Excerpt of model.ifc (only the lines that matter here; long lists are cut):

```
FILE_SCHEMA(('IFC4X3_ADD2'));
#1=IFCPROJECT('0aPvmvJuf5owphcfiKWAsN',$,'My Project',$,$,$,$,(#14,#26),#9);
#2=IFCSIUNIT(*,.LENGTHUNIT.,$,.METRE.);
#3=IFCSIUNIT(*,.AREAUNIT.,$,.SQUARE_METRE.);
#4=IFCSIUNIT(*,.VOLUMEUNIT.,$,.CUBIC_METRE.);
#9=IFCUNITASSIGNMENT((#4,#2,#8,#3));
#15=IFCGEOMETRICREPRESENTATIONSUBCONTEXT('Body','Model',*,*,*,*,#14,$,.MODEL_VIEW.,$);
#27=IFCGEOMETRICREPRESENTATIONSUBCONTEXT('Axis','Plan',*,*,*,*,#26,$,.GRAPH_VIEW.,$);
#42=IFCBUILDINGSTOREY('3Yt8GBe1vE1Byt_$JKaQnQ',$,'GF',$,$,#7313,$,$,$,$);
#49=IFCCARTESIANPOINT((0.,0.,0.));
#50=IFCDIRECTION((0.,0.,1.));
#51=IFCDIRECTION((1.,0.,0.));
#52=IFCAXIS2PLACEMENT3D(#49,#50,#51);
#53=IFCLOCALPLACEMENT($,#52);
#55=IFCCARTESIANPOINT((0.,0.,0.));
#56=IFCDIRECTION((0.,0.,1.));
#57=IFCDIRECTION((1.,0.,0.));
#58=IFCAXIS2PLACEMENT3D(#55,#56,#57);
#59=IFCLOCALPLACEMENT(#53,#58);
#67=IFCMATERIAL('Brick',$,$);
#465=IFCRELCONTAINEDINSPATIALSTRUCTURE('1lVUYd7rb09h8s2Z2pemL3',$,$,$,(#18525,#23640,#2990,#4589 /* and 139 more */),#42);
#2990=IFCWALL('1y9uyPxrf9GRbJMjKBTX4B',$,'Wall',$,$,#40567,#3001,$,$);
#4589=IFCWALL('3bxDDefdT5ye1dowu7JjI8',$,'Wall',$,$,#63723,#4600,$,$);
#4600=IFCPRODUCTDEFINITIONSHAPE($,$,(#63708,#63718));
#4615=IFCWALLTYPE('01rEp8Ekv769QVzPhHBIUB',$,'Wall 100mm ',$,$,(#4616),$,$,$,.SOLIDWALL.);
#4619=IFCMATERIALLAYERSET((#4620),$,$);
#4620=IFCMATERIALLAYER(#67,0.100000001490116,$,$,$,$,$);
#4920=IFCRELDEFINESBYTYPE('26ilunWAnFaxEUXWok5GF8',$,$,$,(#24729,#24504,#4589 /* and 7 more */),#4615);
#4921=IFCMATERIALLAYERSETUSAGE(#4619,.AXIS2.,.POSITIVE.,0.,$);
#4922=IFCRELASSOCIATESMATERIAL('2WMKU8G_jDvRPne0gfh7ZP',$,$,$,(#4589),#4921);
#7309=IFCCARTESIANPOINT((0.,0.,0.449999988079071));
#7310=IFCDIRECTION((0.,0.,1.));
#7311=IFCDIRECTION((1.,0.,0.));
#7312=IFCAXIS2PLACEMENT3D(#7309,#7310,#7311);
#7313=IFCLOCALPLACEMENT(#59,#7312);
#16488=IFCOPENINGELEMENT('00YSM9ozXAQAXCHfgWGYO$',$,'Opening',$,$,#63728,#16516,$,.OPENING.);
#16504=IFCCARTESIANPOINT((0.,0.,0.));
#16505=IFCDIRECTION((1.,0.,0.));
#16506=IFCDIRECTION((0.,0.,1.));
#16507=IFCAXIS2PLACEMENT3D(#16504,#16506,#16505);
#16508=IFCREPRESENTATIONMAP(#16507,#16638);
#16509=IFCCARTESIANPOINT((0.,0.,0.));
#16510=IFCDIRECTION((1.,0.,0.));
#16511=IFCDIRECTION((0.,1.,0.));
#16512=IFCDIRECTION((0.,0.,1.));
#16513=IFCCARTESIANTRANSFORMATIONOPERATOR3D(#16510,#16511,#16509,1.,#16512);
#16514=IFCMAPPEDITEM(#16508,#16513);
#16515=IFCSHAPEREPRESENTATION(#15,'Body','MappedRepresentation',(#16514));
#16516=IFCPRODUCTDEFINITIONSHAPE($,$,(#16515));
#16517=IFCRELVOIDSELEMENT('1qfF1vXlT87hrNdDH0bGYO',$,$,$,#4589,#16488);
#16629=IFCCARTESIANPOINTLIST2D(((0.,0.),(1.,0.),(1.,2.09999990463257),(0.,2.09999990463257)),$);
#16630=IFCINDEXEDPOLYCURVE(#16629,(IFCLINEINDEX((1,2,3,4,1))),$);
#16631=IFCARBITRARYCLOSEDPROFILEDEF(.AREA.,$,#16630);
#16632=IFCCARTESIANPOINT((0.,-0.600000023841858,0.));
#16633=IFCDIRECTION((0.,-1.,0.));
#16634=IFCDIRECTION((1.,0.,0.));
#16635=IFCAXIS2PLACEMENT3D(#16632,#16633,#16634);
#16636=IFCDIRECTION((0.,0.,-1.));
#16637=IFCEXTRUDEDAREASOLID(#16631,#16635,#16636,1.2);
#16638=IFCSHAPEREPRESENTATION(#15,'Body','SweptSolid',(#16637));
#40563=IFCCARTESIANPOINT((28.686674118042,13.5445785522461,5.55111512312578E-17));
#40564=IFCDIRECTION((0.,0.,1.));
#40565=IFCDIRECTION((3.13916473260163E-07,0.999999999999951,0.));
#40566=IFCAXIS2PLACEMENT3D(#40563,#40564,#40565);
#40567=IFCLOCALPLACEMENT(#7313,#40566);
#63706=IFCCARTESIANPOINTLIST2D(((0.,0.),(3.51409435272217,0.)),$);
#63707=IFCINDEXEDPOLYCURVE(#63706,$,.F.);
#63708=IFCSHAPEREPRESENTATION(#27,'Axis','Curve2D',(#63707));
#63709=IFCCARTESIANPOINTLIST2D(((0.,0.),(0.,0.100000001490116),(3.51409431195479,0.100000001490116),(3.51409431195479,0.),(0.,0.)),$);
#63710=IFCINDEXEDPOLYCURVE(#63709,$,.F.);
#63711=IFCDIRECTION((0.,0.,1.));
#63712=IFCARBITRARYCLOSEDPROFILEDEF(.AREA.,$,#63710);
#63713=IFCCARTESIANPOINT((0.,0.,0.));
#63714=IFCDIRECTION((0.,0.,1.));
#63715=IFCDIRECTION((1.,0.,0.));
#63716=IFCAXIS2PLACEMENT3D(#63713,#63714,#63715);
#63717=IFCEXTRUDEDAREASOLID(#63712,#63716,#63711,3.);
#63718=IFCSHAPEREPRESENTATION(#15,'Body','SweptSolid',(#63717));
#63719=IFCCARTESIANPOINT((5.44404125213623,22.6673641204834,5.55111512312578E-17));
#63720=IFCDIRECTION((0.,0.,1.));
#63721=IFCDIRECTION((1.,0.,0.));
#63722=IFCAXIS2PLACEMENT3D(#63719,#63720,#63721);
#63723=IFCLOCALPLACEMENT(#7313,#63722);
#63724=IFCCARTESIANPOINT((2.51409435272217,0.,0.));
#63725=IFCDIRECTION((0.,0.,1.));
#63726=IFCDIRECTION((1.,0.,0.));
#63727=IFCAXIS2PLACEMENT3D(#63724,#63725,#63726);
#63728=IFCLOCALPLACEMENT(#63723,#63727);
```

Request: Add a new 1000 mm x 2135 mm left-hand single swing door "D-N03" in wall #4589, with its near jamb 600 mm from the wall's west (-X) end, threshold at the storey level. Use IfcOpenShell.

```python
import numpy as np
import ifcopenshell
import ifcopenshell.api.feature
import ifcopenshell.api.geometry
import ifcopenshell.api.root
import ifcopenshell.api.spatial
import ifcopenshell.geom
import ifcopenshell.util.element
import ifcopenshell.util.placement
import ifcopenshell.util.representation
import ifcopenshell.util.shape
import ifcopenshell.util.unit

model = ifcopenshell.open("model.ifc")
unit_scale = ifcopenshell.util.unit.calculate_unit_scale(model)
settings = ifcopenshell.geom.settings()


def volume(element):
    """Net volume in cubic metres, openings subtracted."""
    shape = ifcopenshell.geom.create_shape(settings, element)
    return ifcopenshell.util.shape.get_volume(shape.geometry)


wall = model.by_guid("3bxDDefdT5ye1dowu7JjI8")
storey = ifcopenshell.util.element.get_container(wall, ifc_class="IfcBuildingStorey")
context = ifcopenshell.util.representation.get_context(model, "Model", "Body", "MODEL_VIEW")
before = volume(wall)

width, height, from_end, sill = 1, 2.135, 0.6, 0.0  # metres

# The wall runs along its own X axis, and the end named is its -X end.
wall_shape = ifcopenshell.geom.create_shape(settings, wall)
x, y, z = ifcopenshell.util.shape.get_vertices(wall_shape.geometry).T
start = x.min() + from_end
face, thickness = float(y.min()), float(y.max() - y.min())
wall_matrix = ifcopenshell.util.placement.get_local_placement(wall.ObjectPlacement)
level = ifcopenshell.util.placement.get_local_placement(storey.ObjectPlacement)[2, 3]


def in_wall(x, y):
    """Placement at x, y metres in the wall's axes, at sill height."""
    matrix = wall_matrix.copy()
    matrix[:, 3] = wall_matrix @ np.array([x / unit_scale, y / unit_scale, 0.0, 1.0])
    matrix[2, 3] = level + sill / unit_scale
    return matrix


# Opening: a box that overshoots both wall faces by 50 mm.
opening = ifcopenshell.api.root.create_entity(model, ifc_class="IfcOpeningElement", predefined_type="OPENING")
box = ifcopenshell.api.geometry.add_wall_representation(
    model, context=context, length=width, height=height, thickness=thickness + 0.1
)
ifcopenshell.api.geometry.assign_representation(model, product=opening, representation=box)
ifcopenshell.api.geometry.edit_object_placement(model, product=opening, matrix=in_wall(start, face - 0.05), is_si=False)
ifcopenshell.api.feature.add_feature(model, feature=opening, element=wall)

door = ifcopenshell.api.root.create_entity(model, ifc_class="IfcDoor", name="D-N03", predefined_type="DOOR")
door.OverallWidth, door.OverallHeight = width / unit_scale, height / unit_scale
door.OperationType = "SINGLE_SWING_LEFT"
body = ifcopenshell.api.geometry.add_door_representation(
    model,
    context=context,
    overall_width=door.OverallWidth,
    overall_height=door.OverallHeight,
    operation_type="SINGLE_SWING_LEFT",
    lining_properties={"LiningDepth": thickness / unit_scale, "ThresholdDepth": thickness / unit_scale},
)
ifcopenshell.api.geometry.assign_representation(model, product=door, representation=body)
ifcopenshell.api.spatial.assign_container(model, products=[door], relating_structure=storey)
ifcopenshell.api.feature.add_filling(model, opening=opening, element=door)

# The lining spans the wall, so the door starts at the wall face.
ifcopenshell.api.geometry.edit_object_placement(model, product=door, matrix=in_wall(start, face), is_si=False)

after = volume(wall)

print(f"wall volume {before:.3f} -> {after:.3f} m3")

model.write("model_updated.ifc")
```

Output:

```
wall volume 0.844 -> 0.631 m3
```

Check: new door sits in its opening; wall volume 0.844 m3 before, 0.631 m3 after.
